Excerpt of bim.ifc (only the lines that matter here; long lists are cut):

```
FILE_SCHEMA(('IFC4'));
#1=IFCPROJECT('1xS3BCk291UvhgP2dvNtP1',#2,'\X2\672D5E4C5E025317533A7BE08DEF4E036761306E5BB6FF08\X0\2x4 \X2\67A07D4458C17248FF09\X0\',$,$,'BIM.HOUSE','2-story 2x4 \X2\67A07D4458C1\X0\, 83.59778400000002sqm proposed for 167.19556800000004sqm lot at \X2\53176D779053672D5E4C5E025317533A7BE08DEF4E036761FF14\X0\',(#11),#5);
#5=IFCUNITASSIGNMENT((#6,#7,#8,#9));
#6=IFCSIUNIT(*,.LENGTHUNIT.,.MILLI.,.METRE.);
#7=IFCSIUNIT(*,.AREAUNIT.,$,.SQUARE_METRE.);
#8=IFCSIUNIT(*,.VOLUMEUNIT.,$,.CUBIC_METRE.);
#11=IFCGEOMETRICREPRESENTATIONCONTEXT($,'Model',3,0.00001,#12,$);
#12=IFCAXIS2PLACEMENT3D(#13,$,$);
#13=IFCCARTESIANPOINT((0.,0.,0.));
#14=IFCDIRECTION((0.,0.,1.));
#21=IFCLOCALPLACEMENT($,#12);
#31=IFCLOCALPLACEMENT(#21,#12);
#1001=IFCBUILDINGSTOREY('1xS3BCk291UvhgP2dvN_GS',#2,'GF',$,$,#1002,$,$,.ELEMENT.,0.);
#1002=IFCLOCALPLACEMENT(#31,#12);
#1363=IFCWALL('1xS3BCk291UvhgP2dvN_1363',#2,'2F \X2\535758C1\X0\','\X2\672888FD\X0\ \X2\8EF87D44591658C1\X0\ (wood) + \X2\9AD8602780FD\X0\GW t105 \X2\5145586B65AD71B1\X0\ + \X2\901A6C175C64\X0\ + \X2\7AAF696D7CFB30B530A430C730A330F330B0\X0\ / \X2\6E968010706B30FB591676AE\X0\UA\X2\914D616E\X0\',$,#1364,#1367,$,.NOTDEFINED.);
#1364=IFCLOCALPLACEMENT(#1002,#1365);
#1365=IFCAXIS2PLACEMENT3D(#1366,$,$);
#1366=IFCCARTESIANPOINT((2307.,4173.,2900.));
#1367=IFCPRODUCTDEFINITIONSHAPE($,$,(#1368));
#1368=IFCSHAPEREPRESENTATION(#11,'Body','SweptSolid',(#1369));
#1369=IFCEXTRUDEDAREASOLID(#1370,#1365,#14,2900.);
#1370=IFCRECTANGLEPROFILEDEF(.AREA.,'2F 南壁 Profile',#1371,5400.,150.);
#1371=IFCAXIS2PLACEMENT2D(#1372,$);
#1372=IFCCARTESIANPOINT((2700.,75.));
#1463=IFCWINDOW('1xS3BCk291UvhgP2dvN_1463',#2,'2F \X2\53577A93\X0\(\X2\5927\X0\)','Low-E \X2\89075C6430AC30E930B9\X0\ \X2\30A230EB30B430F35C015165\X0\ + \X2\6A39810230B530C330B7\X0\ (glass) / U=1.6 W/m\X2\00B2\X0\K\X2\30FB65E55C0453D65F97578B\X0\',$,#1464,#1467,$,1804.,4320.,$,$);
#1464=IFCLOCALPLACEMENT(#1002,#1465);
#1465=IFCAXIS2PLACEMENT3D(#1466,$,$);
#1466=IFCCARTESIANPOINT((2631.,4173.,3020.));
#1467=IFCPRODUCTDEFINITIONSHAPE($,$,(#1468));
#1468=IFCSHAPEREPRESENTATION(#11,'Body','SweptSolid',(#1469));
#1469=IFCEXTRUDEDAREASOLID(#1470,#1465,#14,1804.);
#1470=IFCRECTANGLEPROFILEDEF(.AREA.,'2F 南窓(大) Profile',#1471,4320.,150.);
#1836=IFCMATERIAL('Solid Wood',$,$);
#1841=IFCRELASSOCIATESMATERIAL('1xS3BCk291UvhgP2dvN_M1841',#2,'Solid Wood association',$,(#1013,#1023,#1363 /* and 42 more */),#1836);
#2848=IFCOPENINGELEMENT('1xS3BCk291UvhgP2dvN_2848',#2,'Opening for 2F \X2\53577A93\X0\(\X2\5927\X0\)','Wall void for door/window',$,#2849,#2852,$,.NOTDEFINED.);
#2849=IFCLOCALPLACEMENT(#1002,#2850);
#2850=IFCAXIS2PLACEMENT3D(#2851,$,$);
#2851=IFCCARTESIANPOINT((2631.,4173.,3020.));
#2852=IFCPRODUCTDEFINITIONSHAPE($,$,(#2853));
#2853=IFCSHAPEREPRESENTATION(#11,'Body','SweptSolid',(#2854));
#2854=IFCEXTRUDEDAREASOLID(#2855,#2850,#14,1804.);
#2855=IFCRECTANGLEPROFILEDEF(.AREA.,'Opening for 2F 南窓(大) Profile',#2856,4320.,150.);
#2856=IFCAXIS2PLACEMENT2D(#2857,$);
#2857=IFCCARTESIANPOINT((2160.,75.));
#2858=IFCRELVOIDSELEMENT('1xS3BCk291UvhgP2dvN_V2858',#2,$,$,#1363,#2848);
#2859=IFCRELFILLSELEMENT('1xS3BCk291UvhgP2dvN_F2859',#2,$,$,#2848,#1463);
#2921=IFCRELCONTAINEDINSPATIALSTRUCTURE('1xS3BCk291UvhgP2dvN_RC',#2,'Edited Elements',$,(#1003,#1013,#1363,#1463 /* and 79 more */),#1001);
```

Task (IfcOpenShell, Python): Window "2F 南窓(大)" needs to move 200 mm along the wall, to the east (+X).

```python
import ifcopenshell
import ifcopenshell.api.geometry
import ifcopenshell.util.placement
import ifcopenshell.util.unit

model = ifcopenshell.open("bim.ifc")
unit_scale = ifcopenshell.util.unit.calculate_unit_scale(model)

window = model.by_guid("1xS3BCk291UvhgP2dvN_1463")
opening = window.FillsVoids[0].RelatingOpeningElement
wall = opening.VoidsElements[0].RelatingBuildingElement

wall_matrix = ifcopenshell.util.placement.get_local_placement(wall.ObjectPlacement)
shift = wall_matrix[:3, 0] * 0.2 / unit_scale
before = ifcopenshell.util.placement.get_local_placement(window.ObjectPlacement)[:3, 3].copy()

# The window is not placed relative to its opening, so move both.
for product in (opening, window):
    matrix = ifcopenshell.util.placement.get_local_placement(product.ObjectPlacement)
    matrix[:3, 3] += shift
    ifcopenshell.api.geometry.edit_object_placement(model, product=product, matrix=matrix, is_si=False)

after = ifcopenshell.util.placement.get_local_placement(window.ObjectPlacement)[:3, 3]
print("window moved by", (after - before).round(3) + 0.0)

model.write("bim_updated.ifc")
```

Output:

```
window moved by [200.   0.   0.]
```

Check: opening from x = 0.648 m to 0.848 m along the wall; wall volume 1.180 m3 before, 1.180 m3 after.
